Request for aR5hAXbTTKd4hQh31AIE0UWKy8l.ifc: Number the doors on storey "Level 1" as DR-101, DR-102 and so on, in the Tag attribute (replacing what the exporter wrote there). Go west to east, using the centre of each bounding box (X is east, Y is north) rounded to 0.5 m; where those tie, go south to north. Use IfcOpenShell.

First a look at what the model holds.

```python
import ifcopenshell
import ifcopenshell.util.element
import ifcopenshell.util.placement

model = ifcopenshell.open("aR5hAXbTTKd4hQh31AIE0UWKy8l.ifc")
print(model.schema)
storey = next(s for s in model.by_type("IfcBuildingStorey") if s.Name == "Level 1")
doors = [e for e in ifcopenshell.util.element.get_decomposition(storey) if e.is_a("IfcDoor")]
for e in sorted(doors, key=lambda e: e.id()):
    origin = ifcopenshell.util.placement.get_local_placement(e.ObjectPlacement)[:3, 3]
    print(e.id(), e.Tag, e.Name, origin.round(2) + 0.0, sep=" | ")
```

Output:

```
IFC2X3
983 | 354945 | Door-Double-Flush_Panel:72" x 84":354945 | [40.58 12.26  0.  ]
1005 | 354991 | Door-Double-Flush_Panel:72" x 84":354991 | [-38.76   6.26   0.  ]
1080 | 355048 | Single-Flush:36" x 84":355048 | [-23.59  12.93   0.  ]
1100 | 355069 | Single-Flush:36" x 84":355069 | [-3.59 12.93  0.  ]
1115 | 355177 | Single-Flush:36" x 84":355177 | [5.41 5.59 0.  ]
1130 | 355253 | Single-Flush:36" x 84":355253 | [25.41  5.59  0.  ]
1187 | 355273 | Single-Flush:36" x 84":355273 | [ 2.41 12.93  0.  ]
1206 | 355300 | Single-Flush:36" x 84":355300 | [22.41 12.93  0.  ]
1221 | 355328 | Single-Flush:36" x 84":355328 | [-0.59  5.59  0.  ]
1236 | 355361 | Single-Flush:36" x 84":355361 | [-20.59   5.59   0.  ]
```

```python
import ifcopenshell
import ifcopenshell.geom
import ifcopenshell.util.element
import ifcopenshell.util.shape

model = ifcopenshell.open("aR5hAXbTTKd4hQh31AIE0UWKy8l.ifc")
settings = ifcopenshell.geom.settings()
settings.set("use-world-coords", True)


def centre(element):
    shape = ifcopenshell.geom.create_shape(settings, element)
    return ifcopenshell.util.shape.get_bbox_centroid(shape.geometry)


storey = next(s for s in model.by_type("IfcBuildingStorey") if s.Name == "Level 1")
doors = [e for e in ifcopenshell.util.element.get_decomposition(storey) if e.is_a("IfcDoor")]

# Insertion points can sit at a corner or the storey origin, so sort by the geometry (in metres).
centres = {e: centre(e) for e in doors}
doors.sort(key=lambda e: (round(centres[e][0] / 0.5), centres[e][1]))

for i, e in enumerate(doors, start=1):
    number = f"DR-1{i:02d}"
    e.Tag = number
    print(e.id(), number)

model.write("aR5hAXbTTKd4hQh31AIE0UWKy8l-out.ifc")
```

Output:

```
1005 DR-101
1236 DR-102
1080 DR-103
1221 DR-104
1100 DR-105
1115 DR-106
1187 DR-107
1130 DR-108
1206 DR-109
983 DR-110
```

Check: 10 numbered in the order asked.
